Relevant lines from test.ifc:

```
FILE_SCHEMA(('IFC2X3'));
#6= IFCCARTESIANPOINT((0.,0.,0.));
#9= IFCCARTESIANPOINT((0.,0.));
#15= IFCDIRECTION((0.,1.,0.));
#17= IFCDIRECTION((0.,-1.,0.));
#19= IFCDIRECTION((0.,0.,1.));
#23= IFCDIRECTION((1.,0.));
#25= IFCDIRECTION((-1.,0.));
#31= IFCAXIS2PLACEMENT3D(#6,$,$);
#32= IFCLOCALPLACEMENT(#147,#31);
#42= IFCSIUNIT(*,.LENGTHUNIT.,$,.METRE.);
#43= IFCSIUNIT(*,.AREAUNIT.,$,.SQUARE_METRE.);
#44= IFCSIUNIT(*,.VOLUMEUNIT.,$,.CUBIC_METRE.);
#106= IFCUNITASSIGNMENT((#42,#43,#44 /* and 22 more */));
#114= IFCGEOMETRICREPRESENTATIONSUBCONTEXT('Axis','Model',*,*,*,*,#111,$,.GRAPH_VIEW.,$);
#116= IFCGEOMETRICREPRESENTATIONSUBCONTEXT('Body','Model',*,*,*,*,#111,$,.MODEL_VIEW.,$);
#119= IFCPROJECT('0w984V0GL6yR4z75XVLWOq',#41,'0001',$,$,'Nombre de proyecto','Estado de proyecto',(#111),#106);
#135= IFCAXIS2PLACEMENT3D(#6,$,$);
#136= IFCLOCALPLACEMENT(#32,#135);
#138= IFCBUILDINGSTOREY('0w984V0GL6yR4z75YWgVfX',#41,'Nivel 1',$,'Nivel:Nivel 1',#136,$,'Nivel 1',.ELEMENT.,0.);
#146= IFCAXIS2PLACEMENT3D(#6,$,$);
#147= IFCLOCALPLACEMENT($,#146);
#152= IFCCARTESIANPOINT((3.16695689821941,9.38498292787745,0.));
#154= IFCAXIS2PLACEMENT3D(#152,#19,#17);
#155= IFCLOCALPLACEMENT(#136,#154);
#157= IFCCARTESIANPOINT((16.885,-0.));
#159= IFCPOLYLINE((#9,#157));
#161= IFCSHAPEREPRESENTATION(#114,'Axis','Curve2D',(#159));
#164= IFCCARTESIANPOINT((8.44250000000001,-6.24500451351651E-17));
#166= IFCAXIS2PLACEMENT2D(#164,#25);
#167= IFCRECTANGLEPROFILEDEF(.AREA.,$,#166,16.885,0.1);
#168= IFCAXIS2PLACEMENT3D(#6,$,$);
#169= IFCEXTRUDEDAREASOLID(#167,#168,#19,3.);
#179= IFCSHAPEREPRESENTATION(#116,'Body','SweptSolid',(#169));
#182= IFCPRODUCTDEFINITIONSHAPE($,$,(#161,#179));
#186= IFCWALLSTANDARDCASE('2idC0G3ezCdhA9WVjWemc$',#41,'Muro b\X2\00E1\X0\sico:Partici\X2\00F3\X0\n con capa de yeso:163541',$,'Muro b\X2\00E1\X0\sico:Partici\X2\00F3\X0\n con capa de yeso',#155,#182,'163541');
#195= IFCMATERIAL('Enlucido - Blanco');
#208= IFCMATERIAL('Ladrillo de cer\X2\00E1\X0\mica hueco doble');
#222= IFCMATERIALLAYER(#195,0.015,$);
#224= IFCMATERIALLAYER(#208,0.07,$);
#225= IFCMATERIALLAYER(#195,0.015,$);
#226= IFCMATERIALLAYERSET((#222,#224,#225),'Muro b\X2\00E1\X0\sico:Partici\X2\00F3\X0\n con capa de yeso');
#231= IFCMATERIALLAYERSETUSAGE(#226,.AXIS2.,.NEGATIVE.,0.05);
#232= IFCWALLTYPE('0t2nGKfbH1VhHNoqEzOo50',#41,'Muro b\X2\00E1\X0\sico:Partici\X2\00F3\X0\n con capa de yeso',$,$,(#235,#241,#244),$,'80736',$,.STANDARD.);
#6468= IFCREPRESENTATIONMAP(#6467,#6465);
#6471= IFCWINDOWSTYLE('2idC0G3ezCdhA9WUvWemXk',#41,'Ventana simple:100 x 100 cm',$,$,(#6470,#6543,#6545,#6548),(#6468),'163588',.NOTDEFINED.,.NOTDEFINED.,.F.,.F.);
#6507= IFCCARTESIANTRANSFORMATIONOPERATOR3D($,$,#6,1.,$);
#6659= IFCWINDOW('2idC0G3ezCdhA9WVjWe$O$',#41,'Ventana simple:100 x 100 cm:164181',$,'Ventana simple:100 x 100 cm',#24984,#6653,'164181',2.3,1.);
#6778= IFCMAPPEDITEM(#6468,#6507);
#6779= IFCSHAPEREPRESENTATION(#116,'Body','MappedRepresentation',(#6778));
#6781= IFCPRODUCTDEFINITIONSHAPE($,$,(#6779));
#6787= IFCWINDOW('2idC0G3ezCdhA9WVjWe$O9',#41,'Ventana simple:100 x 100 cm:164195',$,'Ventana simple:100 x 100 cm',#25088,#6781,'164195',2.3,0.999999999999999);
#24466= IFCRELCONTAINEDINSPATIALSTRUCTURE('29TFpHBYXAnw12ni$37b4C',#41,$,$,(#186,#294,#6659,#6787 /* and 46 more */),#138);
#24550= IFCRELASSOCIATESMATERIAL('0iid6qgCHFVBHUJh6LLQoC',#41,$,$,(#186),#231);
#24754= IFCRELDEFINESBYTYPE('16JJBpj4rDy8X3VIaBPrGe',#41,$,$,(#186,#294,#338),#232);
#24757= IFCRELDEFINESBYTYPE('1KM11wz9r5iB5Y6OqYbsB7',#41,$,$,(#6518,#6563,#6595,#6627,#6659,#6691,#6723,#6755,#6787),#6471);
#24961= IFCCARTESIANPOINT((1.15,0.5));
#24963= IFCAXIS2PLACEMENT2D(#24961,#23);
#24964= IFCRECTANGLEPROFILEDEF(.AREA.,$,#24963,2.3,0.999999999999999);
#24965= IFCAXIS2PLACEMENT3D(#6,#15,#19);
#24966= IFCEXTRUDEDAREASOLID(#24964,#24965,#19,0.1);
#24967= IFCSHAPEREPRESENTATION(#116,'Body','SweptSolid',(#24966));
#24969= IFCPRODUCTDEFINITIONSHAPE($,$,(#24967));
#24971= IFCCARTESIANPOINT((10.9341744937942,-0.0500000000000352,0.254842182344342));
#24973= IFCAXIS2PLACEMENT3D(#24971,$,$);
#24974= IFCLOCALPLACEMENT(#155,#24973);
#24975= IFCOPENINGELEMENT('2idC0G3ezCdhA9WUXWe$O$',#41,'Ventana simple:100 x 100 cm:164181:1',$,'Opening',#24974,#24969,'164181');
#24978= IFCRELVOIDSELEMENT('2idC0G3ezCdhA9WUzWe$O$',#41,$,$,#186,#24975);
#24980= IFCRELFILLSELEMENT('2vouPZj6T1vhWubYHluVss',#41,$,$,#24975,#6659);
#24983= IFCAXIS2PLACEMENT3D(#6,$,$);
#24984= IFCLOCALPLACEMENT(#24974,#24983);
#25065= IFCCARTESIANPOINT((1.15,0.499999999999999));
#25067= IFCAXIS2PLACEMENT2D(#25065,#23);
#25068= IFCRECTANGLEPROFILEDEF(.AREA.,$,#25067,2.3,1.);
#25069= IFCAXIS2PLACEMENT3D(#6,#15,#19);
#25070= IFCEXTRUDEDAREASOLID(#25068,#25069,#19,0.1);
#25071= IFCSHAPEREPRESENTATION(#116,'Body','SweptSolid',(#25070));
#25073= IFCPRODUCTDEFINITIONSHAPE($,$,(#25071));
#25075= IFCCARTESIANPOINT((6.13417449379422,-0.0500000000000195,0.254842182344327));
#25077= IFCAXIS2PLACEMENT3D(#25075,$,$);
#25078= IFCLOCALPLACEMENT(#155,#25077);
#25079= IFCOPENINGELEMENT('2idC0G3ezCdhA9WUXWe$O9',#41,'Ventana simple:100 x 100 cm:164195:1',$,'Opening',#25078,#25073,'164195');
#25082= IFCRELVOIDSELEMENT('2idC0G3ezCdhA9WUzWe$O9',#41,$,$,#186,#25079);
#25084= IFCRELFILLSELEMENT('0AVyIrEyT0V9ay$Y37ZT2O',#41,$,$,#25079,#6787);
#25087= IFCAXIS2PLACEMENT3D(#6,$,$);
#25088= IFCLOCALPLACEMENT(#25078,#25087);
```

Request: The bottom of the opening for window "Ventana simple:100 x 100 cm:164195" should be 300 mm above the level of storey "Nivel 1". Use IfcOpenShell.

```python
import numpy as np
import ifcopenshell
import ifcopenshell.api.geometry
import ifcopenshell.geom
import ifcopenshell.util.element
import ifcopenshell.util.placement
import ifcopenshell.util.shape
import ifcopenshell.util.unit

model = ifcopenshell.open("test.ifc")
unit_scale = ifcopenshell.util.unit.calculate_unit_scale(model)

window = model.by_guid("2idC0G3ezCdhA9WVjWe$O9")
opening = window.FillsVoids[0].RelatingOpeningElement
storey = ifcopenshell.util.element.get_container(window, ifc_class="IfcBuildingStorey")
level = ifcopenshell.util.placement.get_local_placement(storey.ObjectPlacement)[2, 3]

# The opening's origin need not be at the sill, so measure its lowest point.
shape = ifcopenshell.geom.create_shape(ifcopenshell.geom.settings(), opening)
bottom = ifcopenshell.util.shape.get_shape_bottom_elevation(shape, shape.geometry) / unit_scale
dz = level + 0.3 / unit_scale - bottom

shift = np.array([0.0, 0.0, dz])
# The window is placed relative to its opening, so it follows when the opening moves.
matrix = ifcopenshell.util.placement.get_local_placement(opening.ObjectPlacement)
matrix[:3, 3] += shift
ifcopenshell.api.geometry.edit_object_placement(
    model, product=opening, matrix=matrix, is_si=False, should_transform_children=True
)

print(f"moved by {dz * unit_scale:+.3f} m")

model.write("test-out.ifc")
```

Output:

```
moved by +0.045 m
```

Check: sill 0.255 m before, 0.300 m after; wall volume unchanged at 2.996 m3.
